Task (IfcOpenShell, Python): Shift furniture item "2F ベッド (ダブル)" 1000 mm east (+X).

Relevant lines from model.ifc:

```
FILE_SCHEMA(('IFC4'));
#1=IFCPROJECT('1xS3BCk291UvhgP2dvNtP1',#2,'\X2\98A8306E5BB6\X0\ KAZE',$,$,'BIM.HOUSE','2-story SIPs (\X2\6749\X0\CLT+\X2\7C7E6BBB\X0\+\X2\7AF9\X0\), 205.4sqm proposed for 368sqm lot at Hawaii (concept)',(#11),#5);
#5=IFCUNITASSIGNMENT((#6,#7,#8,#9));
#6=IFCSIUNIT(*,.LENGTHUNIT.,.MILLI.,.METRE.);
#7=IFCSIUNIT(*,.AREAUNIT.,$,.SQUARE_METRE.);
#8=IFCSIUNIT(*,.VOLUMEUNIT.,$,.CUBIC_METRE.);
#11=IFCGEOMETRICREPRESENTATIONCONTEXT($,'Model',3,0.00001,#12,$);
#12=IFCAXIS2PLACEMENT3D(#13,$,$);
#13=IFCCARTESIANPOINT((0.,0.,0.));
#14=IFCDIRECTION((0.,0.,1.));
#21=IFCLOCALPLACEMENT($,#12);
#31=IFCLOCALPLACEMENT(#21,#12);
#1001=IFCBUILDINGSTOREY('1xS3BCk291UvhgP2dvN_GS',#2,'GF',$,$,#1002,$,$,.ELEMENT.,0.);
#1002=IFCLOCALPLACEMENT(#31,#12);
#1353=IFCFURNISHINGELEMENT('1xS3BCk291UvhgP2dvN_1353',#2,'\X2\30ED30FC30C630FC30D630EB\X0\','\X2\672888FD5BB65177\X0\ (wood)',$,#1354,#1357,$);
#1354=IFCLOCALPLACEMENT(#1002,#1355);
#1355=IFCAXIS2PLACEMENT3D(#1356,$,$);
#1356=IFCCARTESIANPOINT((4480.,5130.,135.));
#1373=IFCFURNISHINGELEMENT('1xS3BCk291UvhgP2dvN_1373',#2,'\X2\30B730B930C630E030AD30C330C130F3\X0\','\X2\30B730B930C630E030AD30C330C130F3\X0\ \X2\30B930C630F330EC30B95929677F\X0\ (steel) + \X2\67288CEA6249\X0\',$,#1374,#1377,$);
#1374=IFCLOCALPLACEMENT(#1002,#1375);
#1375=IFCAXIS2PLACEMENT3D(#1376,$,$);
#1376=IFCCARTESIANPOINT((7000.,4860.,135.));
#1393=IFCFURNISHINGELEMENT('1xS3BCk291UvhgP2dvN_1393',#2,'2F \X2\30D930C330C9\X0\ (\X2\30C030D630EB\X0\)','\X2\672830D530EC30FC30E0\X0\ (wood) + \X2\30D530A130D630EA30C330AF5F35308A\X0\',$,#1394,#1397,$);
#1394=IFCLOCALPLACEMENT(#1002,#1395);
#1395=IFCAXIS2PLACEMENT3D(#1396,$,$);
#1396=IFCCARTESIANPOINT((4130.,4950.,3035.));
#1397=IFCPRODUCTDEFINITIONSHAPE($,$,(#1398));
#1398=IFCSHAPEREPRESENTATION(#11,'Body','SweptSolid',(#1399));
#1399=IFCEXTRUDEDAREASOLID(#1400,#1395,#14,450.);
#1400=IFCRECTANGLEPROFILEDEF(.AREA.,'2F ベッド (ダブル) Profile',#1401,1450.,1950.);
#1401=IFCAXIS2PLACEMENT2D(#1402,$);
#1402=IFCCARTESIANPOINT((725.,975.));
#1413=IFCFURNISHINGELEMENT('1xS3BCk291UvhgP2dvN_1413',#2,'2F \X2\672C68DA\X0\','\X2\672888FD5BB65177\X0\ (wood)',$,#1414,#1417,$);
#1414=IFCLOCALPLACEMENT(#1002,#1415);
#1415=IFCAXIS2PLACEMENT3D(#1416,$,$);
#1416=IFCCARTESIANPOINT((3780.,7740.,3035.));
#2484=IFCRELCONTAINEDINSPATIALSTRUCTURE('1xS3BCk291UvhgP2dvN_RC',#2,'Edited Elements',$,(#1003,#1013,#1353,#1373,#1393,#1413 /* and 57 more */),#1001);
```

```python
import ifcopenshell
import ifcopenshell.api.geometry
import ifcopenshell.util.placement
import ifcopenshell.util.unit

model = ifcopenshell.open("model.ifc")
unit_scale = ifcopenshell.util.unit.calculate_unit_scale(model)

item = model.by_guid("1xS3BCk291UvhgP2dvN_1393")
matrix = ifcopenshell.util.placement.get_local_placement(item.ObjectPlacement)
matrix[0, 3] += 1 / unit_scale
ifcopenshell.api.geometry.edit_object_placement(model, product=item, matrix=matrix, is_si=False)

print(ifcopenshell.util.placement.get_local_placement(item.ObjectPlacement).round(3) + 0.0)

model.write("model-out.ifc")
```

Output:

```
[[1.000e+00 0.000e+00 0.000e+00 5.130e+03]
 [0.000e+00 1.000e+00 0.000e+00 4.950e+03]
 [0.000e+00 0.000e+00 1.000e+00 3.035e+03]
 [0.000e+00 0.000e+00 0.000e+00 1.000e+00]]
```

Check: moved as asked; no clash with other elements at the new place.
